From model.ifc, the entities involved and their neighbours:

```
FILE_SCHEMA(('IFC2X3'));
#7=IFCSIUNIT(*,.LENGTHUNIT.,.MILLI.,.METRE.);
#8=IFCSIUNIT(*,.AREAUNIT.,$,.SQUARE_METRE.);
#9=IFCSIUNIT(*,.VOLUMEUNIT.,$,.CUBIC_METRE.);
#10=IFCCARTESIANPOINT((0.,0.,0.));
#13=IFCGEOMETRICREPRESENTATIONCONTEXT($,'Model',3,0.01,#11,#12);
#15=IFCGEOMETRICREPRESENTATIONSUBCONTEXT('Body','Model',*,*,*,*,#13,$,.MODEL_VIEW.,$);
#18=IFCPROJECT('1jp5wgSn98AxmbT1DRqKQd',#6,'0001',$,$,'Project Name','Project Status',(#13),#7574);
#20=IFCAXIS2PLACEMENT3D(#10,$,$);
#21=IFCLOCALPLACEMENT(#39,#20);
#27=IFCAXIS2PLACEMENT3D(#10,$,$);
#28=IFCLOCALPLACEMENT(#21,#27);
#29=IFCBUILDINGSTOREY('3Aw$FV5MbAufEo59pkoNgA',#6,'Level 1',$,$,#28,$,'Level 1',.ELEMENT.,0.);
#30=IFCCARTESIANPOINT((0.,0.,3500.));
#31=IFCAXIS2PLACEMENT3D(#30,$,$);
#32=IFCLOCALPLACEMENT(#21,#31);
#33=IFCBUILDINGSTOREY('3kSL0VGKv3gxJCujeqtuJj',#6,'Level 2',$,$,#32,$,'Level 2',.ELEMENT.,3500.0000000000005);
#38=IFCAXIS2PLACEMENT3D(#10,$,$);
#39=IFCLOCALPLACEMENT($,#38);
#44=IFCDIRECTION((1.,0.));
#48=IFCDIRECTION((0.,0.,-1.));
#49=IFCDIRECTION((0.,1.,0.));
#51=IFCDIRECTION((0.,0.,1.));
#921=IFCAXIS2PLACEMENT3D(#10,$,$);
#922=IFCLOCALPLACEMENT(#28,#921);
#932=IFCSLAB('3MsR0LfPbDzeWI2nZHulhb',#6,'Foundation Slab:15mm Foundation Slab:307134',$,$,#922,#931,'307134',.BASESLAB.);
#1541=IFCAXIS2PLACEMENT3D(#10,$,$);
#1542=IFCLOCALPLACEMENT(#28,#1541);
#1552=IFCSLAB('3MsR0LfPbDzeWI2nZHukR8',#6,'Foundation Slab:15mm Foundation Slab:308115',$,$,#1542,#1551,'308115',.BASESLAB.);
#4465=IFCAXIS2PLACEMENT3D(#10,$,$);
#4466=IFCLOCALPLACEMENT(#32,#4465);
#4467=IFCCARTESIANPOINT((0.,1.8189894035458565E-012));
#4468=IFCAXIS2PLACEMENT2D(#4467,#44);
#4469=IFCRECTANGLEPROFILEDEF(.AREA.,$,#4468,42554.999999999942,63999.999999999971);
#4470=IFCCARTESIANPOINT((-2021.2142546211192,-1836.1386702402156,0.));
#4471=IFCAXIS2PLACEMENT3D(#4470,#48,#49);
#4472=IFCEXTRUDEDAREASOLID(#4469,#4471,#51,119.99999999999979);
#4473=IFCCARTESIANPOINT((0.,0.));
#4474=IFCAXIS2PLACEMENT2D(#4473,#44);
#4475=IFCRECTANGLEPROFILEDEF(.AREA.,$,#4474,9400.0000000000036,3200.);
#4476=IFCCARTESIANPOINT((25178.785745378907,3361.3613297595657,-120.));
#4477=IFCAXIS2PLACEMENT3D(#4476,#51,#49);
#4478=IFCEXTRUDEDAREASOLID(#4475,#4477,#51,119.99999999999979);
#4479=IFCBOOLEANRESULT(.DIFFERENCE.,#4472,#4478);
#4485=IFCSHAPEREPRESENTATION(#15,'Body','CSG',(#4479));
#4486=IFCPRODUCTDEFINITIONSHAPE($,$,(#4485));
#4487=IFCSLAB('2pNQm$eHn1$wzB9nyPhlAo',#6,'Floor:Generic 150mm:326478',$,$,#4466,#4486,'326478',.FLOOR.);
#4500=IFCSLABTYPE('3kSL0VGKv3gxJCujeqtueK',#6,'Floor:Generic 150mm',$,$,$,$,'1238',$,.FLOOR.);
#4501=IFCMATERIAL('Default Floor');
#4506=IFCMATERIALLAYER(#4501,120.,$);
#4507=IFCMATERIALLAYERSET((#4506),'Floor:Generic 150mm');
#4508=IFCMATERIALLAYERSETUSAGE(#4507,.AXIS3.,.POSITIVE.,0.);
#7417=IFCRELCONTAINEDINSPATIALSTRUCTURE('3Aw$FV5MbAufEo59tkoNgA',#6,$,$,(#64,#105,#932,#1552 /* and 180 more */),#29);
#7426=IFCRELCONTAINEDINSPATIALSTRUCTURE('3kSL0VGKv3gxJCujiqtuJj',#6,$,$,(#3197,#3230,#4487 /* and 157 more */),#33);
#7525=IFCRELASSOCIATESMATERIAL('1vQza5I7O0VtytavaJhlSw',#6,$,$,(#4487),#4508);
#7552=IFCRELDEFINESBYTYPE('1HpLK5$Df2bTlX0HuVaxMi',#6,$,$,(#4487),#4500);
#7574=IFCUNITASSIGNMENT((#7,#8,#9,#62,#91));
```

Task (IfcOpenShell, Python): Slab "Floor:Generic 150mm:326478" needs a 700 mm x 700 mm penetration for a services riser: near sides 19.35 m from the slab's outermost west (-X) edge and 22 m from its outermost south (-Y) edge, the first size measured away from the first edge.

```python
import numpy as np
import ifcopenshell
import ifcopenshell.api.feature
import ifcopenshell.api.geometry
import ifcopenshell.api.root
import ifcopenshell.geom
import ifcopenshell.util.placement
import ifcopenshell.util.representation
import ifcopenshell.util.shape
import ifcopenshell.util.unit

model = ifcopenshell.open("model.ifc")
unit_scale = ifcopenshell.util.unit.calculate_unit_scale(model)
settings = ifcopenshell.geom.settings()


def volume(element):
    """Net volume in cubic metres, openings subtracted."""
    shape = ifcopenshell.geom.create_shape(settings, element)
    return ifcopenshell.util.shape.get_volume(shape.geometry)


slab = model.by_id(4487)
before = volume(slab)

# Extent in the slab's own axes, in metres. The edges named are its -X and -Y sides.
slab_shape = ifcopenshell.geom.create_shape(settings, slab)
vertices = ifcopenshell.util.shape.get_vertices(slab_shape.geometry)
x_min, y_min, bottom = vertices.min(axis=0)
top = vertices[:, 2].max()

opening = ifcopenshell.api.root.create_entity(model, ifc_class="IfcOpeningElement", name="Services riser opening")
context = ifcopenshell.util.representation.get_context(model, "Model", "Body", "MODEL_VIEW")
width, depth = 0.7, 0.7
outline = [(0.0, 0.0), (width, 0.0), (width, depth), (0.0, depth), (0.0, 0.0)]
# Overshoot both faces by 50 mm so the cut is clean.
shape = ifcopenshell.api.geometry.add_slab_representation(
    model, context=context, depth=top - bottom + 0.1, polyline=outline
)
ifcopenshell.api.geometry.assign_representation(model, product=opening, representation=shape)

matrix = ifcopenshell.util.placement.get_local_placement(slab.ObjectPlacement)
matrix[:, 3] = matrix @ np.append(np.array([x_min + 19.35, y_min + 22, bottom - 0.05]) / unit_scale, 1.0)
ifcopenshell.api.geometry.edit_object_placement(model, product=opening, matrix=matrix, is_si=False)
ifcopenshell.api.feature.add_feature(model, feature=opening, element=slab)

after = volume(slab)

print(f"slab volume {before:.3f} -> {after:.3f} m3")

model.write("model_rev.ifc")
```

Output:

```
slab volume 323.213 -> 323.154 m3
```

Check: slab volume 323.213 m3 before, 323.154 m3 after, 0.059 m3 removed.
